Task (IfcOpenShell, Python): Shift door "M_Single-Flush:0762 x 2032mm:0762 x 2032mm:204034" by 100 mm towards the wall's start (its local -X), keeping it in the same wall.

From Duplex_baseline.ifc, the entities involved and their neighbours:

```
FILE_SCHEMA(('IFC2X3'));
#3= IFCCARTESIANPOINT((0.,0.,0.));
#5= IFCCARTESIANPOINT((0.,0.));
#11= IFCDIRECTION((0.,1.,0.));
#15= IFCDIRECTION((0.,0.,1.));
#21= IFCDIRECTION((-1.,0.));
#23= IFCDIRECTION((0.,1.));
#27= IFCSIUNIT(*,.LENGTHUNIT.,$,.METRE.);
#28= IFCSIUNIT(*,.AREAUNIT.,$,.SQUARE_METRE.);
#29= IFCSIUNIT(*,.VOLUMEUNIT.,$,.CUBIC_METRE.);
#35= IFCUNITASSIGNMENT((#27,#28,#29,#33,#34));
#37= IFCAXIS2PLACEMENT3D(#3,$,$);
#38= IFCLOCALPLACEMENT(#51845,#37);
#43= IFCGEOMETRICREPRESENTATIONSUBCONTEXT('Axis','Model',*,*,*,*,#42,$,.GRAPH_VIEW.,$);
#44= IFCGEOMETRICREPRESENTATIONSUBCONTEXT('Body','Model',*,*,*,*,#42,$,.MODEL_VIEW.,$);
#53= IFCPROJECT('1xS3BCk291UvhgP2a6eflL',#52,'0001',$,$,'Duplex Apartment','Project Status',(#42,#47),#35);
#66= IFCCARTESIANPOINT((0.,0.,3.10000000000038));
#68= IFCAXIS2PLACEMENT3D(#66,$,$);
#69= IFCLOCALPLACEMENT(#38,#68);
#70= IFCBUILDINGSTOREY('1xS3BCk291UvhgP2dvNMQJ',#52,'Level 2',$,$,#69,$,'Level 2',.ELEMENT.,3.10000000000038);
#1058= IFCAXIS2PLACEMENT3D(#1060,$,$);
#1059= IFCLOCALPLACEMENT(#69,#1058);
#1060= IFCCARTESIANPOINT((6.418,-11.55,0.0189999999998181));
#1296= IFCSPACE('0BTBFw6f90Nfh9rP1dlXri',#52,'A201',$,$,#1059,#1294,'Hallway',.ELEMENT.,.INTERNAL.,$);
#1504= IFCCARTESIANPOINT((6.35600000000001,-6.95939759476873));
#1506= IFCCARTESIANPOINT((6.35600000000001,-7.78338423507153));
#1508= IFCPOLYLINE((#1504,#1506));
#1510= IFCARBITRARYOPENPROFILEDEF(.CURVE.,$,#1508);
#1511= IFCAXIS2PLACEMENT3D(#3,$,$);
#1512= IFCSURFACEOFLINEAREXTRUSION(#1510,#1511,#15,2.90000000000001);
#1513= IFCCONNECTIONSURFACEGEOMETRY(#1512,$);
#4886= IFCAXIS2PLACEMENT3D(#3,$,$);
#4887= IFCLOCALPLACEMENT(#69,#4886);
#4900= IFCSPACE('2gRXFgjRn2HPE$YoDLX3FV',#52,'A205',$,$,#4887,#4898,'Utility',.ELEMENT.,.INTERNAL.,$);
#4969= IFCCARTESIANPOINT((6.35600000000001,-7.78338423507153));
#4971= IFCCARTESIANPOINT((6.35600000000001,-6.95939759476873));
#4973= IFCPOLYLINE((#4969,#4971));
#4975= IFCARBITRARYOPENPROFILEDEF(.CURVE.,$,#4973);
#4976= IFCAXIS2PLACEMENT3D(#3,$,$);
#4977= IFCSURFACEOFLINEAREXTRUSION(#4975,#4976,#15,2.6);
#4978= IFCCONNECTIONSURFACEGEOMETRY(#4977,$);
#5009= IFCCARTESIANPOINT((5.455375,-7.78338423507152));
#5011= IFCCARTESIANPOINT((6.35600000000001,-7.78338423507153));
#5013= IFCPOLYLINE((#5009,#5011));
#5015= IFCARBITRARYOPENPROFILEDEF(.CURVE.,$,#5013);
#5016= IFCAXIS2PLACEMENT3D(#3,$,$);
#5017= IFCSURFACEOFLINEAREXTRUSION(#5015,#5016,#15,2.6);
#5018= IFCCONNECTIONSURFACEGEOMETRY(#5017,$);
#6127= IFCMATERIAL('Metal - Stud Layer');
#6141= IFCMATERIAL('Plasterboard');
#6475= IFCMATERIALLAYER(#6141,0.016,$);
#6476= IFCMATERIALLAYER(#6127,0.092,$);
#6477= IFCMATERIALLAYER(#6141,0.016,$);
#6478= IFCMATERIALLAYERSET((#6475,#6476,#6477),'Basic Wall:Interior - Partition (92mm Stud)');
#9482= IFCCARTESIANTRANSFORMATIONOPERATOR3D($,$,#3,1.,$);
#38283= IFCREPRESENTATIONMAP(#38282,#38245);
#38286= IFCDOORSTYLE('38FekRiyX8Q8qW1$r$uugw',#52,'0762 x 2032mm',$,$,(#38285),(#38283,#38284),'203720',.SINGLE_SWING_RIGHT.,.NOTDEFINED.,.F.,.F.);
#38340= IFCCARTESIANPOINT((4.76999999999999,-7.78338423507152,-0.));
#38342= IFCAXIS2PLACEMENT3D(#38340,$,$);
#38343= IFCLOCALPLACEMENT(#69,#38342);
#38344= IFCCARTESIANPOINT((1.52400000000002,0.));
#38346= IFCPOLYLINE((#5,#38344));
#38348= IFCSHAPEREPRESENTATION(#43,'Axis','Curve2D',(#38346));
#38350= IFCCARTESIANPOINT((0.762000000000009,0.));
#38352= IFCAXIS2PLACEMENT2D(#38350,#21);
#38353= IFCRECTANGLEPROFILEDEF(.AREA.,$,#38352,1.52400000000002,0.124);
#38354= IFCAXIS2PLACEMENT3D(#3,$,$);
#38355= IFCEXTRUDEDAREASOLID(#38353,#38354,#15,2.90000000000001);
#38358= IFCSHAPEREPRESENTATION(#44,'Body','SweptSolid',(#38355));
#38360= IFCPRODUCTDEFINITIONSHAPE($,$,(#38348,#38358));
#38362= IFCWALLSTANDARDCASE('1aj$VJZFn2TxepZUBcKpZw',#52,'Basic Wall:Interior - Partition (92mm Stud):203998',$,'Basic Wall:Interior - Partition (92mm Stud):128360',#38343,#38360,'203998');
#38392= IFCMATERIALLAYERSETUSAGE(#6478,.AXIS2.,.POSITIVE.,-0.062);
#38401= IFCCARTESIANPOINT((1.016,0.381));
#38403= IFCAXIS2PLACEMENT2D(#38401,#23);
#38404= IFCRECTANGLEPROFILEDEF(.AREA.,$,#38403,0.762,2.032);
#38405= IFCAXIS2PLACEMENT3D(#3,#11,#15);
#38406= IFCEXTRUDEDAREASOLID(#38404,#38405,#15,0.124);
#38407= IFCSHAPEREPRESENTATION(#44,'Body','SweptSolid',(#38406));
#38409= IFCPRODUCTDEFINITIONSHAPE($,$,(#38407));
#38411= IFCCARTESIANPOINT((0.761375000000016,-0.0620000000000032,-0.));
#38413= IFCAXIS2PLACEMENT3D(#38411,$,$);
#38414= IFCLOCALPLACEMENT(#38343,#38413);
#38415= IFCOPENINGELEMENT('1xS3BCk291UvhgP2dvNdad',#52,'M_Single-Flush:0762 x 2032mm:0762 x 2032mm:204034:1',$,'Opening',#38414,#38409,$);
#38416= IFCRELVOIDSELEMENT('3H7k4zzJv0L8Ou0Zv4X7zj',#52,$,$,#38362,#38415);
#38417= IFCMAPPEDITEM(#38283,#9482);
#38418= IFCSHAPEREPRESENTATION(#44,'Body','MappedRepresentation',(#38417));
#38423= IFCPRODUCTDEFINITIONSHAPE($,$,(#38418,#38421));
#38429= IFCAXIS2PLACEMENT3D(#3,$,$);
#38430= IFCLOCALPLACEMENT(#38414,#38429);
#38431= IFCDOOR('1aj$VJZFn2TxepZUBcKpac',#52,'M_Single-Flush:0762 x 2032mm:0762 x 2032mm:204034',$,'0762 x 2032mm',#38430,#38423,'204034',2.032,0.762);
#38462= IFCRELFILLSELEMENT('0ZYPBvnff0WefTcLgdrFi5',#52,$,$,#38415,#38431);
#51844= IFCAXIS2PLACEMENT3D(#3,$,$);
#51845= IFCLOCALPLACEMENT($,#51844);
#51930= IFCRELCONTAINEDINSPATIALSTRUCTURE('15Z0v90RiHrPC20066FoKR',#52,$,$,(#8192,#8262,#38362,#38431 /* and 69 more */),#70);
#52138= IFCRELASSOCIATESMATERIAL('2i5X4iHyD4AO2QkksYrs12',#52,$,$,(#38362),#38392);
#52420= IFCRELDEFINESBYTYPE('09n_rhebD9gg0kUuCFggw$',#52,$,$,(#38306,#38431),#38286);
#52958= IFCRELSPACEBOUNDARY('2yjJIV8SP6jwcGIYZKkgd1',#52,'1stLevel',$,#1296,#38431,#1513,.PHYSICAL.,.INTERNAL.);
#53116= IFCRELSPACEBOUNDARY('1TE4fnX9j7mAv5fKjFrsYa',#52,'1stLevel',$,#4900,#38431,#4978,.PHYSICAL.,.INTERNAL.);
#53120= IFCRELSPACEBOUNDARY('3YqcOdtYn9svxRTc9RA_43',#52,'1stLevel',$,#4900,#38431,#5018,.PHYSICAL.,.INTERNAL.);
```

```python
import numpy as np
import ifcopenshell
import ifcopenshell.api.geometry
import ifcopenshell.util.placement
import ifcopenshell.util.unit

model = ifcopenshell.open("Duplex_baseline.ifc")
unit_scale = ifcopenshell.util.unit.calculate_unit_scale(model)

door = model.by_guid("1aj$VJZFn2TxepZUBcKpac")
opening = door.FillsVoids[0].RelatingOpeningElement
wall = opening.VoidsElements[0].RelatingBuildingElement

wall_matrix = ifcopenshell.util.placement.get_local_placement(wall.ObjectPlacement)
shift = wall_matrix[:3, 0] * -0.1 / unit_scale
before = ifcopenshell.util.placement.get_local_placement(door.ObjectPlacement)[:3, 3].copy()

# The door is placed relative to its opening, so it follows when the opening moves.
matrix = ifcopenshell.util.placement.get_local_placement(opening.ObjectPlacement)
matrix[:3, 3] += shift
ifcopenshell.api.geometry.edit_object_placement(
    model, product=opening, matrix=matrix, is_si=False, should_transform_children=True
)

# Space boundary surfaces are stored in each space's coordinates; move them too.
for rel in door.ProvidesBoundaries:
    if not rel.ConnectionGeometry:
        continue
    surface = rel.ConnectionGeometry.SurfaceOnRelatingElement
    space_matrix = ifcopenshell.util.placement.get_local_placement(rel.RelatingSpace.ObjectPlacement)
    point = np.array(surface.Position.Location.Coordinates) + space_matrix[:3, :3].T @ shift
    surface.Position = model.createIfcAxis2Placement3D(
        model.createIfcCartesianPoint(point.tolist()), surface.Position.Axis, surface.Position.RefDirection
    )

after = ifcopenshell.util.placement.get_local_placement(door.ObjectPlacement)[:3, 3]
print("door moved by", (after - before).round(3) + 0.0)

model.write("Duplex_baseline_rev.ifc")
```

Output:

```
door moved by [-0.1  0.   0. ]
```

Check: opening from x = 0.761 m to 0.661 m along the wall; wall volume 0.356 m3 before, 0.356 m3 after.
